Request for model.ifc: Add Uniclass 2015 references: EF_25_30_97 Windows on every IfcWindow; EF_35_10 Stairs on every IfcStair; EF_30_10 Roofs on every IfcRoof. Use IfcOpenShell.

First a look at what the model holds.

```python
import ifcopenshell

model = ifcopenshell.open("model.ifc")
print(model.schema)
print("classifications:", [c.Name for c in model.by_type("IfcClassification")])
for ifc_class in ("IfcDoor", "IfcRoof", "IfcStair", "IfcWall", "IfcWindow"):
    print(ifc_class, len(model.by_type(ifc_class)))
```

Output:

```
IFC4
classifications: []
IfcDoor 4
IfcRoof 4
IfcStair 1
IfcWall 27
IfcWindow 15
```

```python
import ifcopenshell
import ifcopenshell.api.classification

model = ifcopenshell.open("model.ifc")

system = ifcopenshell.api.classification.add_classification(model, classification="Uniclass 2015")

codes = {
    "IfcWindow": ("EF_25_30_97", "Windows"),
    "IfcStair": ("EF_35_10", "Stairs"),
    "IfcRoof": ("EF_30_10", "Roofs"),
}
for ifc_class, (code, name) in codes.items():
    products = model.by_type(ifc_class)
    ifcopenshell.api.classification.add_reference(
        model, products=products, classification=system, identification=code, name=name
    )
    print(code, len(products))

model.write("model-out.ifc")
```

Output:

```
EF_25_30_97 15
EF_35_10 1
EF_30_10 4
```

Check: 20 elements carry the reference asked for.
